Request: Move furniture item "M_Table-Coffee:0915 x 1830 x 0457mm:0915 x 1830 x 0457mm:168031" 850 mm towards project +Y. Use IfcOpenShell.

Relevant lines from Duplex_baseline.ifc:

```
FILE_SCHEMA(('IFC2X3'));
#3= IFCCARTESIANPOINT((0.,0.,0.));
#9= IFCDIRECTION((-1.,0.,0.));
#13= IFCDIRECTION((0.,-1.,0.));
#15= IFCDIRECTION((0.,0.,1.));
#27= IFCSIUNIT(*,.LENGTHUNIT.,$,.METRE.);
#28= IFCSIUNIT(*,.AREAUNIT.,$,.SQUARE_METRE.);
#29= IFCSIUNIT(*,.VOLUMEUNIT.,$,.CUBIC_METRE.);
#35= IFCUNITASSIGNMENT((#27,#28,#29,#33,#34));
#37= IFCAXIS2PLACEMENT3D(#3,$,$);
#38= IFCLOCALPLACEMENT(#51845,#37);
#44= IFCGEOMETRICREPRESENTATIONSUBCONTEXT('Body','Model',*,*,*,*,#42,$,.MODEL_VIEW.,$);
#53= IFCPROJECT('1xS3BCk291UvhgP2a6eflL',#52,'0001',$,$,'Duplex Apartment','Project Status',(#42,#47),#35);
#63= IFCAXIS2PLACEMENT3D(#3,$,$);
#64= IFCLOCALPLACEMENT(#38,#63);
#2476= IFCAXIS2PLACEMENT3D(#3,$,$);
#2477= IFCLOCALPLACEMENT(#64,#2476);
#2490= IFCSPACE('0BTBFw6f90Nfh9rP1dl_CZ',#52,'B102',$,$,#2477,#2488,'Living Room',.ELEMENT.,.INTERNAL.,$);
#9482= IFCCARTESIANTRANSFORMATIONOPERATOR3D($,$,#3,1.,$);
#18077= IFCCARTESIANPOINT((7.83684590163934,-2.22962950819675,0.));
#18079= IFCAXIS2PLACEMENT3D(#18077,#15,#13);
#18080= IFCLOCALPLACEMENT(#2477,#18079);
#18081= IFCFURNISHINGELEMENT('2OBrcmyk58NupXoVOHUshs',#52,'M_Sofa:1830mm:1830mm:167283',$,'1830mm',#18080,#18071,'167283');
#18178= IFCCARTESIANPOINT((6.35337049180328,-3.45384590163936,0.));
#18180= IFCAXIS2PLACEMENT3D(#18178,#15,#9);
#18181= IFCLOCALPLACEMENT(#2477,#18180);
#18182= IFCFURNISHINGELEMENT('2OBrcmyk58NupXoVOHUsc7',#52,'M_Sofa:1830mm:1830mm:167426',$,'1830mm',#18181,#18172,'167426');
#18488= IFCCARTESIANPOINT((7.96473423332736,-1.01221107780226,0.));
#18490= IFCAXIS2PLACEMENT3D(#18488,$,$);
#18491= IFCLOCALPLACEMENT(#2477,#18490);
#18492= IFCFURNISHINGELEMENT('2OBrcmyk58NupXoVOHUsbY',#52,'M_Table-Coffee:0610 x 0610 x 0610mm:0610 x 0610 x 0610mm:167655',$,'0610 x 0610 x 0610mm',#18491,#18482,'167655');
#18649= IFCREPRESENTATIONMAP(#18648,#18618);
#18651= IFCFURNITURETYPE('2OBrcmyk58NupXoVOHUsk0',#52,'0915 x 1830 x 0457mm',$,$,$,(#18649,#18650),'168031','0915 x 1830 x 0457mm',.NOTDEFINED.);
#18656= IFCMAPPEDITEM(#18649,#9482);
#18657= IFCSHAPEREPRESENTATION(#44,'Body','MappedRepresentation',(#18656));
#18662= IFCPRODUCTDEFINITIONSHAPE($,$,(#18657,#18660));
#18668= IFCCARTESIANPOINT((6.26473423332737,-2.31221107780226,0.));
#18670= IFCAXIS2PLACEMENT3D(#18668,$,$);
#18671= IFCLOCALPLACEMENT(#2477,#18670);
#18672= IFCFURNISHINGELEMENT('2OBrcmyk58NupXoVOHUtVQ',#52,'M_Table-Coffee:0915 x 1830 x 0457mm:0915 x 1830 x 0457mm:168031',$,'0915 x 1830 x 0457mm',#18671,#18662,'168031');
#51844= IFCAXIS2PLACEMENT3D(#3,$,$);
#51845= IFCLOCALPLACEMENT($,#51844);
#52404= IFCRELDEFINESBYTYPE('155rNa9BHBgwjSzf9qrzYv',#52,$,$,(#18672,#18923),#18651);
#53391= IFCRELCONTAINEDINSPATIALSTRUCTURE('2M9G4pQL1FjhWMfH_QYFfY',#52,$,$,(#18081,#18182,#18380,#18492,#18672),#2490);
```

```python
import ifcopenshell
import ifcopenshell.api.geometry
import ifcopenshell.util.placement
import ifcopenshell.util.unit

model = ifcopenshell.open("Duplex_baseline.ifc")
unit_scale = ifcopenshell.util.unit.calculate_unit_scale(model)

item = model.by_id(18672)
matrix = ifcopenshell.util.placement.get_local_placement(item.ObjectPlacement)
matrix[1, 3] += 0.85 / unit_scale
ifcopenshell.api.geometry.edit_object_placement(model, product=item, matrix=matrix, is_si=False)

print(ifcopenshell.util.placement.get_local_placement(item.ObjectPlacement).round(3) + 0.0)

model.write("Duplex_baseline_rev.ifc")
```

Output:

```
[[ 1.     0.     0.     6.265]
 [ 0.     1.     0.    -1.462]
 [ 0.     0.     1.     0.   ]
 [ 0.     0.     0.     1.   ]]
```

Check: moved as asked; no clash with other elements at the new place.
